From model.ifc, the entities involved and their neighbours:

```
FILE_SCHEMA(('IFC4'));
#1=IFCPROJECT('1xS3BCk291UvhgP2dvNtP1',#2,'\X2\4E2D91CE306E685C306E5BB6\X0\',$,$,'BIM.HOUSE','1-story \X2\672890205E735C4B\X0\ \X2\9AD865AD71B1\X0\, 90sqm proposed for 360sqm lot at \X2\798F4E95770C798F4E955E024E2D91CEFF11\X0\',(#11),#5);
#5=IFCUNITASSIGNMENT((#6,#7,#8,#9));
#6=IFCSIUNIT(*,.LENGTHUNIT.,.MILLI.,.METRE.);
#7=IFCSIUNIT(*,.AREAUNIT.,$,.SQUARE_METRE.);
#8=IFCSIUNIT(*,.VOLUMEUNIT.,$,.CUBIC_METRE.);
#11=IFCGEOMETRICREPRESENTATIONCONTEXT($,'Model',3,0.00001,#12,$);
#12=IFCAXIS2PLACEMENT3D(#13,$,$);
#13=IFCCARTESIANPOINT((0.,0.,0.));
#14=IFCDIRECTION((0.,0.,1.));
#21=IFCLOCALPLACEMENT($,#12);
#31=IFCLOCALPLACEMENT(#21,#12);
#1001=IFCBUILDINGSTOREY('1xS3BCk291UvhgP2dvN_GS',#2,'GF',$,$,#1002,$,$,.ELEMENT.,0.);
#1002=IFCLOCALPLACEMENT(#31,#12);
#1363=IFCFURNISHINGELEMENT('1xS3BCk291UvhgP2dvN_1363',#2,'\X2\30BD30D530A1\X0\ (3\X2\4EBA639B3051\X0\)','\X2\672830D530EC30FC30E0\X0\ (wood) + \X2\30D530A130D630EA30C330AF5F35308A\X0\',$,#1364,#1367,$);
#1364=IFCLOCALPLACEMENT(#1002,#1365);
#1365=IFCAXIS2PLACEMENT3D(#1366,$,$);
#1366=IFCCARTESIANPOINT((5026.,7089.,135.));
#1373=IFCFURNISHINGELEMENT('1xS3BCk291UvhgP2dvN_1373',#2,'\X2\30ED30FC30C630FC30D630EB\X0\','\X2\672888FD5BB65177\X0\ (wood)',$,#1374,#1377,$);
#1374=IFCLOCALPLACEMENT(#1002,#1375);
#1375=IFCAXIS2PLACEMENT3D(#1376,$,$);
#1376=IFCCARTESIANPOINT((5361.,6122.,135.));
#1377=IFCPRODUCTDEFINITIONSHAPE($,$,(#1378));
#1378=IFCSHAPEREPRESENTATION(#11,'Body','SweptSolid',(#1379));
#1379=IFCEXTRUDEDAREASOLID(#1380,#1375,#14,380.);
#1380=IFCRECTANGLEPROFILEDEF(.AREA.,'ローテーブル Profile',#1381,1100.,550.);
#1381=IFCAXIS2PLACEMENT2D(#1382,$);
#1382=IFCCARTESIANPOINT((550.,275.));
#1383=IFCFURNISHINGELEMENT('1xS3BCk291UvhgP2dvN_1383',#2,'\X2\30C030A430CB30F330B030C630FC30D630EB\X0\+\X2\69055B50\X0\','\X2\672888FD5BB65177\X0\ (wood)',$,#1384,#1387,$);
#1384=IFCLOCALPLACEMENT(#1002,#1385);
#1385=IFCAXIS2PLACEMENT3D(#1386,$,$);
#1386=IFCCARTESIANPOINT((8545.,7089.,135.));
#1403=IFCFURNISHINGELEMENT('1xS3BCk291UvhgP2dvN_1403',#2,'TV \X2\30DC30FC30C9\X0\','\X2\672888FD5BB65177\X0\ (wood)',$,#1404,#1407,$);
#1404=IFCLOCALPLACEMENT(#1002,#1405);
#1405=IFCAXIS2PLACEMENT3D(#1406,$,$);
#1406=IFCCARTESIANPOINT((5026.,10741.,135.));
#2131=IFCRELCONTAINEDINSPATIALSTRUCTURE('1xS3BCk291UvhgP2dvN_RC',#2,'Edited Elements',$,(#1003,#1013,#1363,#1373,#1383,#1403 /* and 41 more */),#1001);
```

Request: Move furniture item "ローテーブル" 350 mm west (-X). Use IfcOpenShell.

```python
import ifcopenshell
import ifcopenshell.api.geometry
import ifcopenshell.util.placement
import ifcopenshell.util.unit

model = ifcopenshell.open("model.ifc")
unit_scale = ifcopenshell.util.unit.calculate_unit_scale(model)

item = model.by_guid("1xS3BCk291UvhgP2dvN_1373")
matrix = ifcopenshell.util.placement.get_local_placement(item.ObjectPlacement)
matrix[0, 3] -= 0.35 / unit_scale
ifcopenshell.api.geometry.edit_object_placement(model, product=item, matrix=matrix, is_si=False)

print(ifcopenshell.util.placement.get_local_placement(item.ObjectPlacement).round(3) + 0.0)

model.write("model_edited.ifc")
```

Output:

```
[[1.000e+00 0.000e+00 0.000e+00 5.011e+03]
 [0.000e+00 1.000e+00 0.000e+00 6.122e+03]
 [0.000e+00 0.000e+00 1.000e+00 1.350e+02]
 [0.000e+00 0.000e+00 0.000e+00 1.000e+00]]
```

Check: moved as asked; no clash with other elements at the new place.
